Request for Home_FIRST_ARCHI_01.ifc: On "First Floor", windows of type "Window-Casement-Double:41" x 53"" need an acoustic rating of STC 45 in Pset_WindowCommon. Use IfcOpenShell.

First a look at what the model holds.

```python
import ifcopenshell
import ifcopenshell.util.element

model = ifcopenshell.open("Home_FIRST_ARCHI_01.ifc")
print(model.schema)
storey = next(s for s in model.by_type("IfcBuildingStorey") if s.Name == "First Floor")
windows = [e for e in ifcopenshell.util.element.get_decomposition(storey) if e.is_a("IfcWindow")]
seen = {}
for e in windows:
    element_type = ifcopenshell.util.element.get_type(e)
    key = (element_type.Name if element_type != e and element_type else None, ifcopenshell.util.element.get_pset(e, "Pset_WindowCommon", "AcousticRating"))
    seen[key] = seen.get(key, 0) + 1
for (name, value), count in sorted(seen.items(), key=str):
    print(count, "x", name, "|", value)
```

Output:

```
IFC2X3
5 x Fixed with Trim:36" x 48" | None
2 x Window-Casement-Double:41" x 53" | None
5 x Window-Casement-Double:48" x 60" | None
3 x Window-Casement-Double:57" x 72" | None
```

```python
import ifcopenshell
import ifcopenshell.api.pset
import ifcopenshell.util.element

model = ifcopenshell.open("Home_FIRST_ARCHI_01.ifc")

storey = next(s for s in model.by_type("IfcBuildingStorey") if s.Name == "First Floor")
windows = [e for e in ifcopenshell.util.element.get_decomposition(storey) if e.is_a("IfcWindow")]

count = 0
for e in windows:
    element_type = ifcopenshell.util.element.get_type(e)
    if element_type in (None, e) or element_type.Name != 'Window-Casement-Double:41" x 53"':
        continue
    # add_pset returns the element's existing set when there is one.
    pset = ifcopenshell.api.pset.add_pset(model, product=e, name="Pset_WindowCommon")
    ifcopenshell.api.pset.edit_pset(model, pset=pset, properties={"AcousticRating": "STC 45"})
    count += 1

print(count, "windows updated")

model.write("Home_FIRST_ARCHI_01_updated.ifc")
```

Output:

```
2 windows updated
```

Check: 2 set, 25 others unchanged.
